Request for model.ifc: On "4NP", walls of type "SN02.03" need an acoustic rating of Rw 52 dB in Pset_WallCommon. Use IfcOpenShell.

First a look at what the model holds.

```python
import ifcopenshell
import ifcopenshell.util.element

model = ifcopenshell.open("model.ifc")
print(model.schema)
storey = next(s for s in model.by_type("IfcBuildingStorey") if s.Name == "4NP")
walls = [e for e in ifcopenshell.util.element.get_decomposition(storey) if e.is_a("IfcWall")]
seen = {}
for e in walls:
    element_type = ifcopenshell.util.element.get_type(e)
    key = (element_type.Name if element_type != e and element_type else None, ifcopenshell.util.element.get_pset(e, "Pset_WallCommon", "AcousticRating"))
    seen[key] = seen.get(key, 0) + 1
for (name, value), count in sorted(seen.items(), key=str):
    print(count, "x", name, "|", value)
```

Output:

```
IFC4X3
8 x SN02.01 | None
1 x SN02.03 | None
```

```python
import ifcopenshell
import ifcopenshell.api.pset
import ifcopenshell.util.element

model = ifcopenshell.open("model.ifc")

storey = next(s for s in model.by_type("IfcBuildingStorey") if s.Name == "4NP")
walls = [e for e in ifcopenshell.util.element.get_decomposition(storey) if e.is_a("IfcWall")]

count = 0
for e in walls:
    element_type = ifcopenshell.util.element.get_type(e)
    if element_type in (None, e) or element_type.Name != "SN02.03":
        continue
    # add_pset returns the element's existing set when there is one.
    pset = ifcopenshell.api.pset.add_pset(model, product=e, name="Pset_WallCommon")
    ifcopenshell.api.pset.edit_pset(model, pset=pset, properties={"AcousticRating": "Rw 52 dB"})
    count += 1

print(count, "walls updated")

model.write("model_edited.ifc")
```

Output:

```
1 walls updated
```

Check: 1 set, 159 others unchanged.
